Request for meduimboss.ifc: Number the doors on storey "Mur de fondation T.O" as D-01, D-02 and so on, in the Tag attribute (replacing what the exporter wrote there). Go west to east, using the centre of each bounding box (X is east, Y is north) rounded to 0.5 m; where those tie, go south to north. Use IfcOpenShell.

First a look at what the model holds.

```python
import ifcopenshell
import ifcopenshell.util.element
import ifcopenshell.util.placement

model = ifcopenshell.open("meduimboss.ifc")
print(model.schema)
storey = next(s for s in model.by_type("IfcBuildingStorey") if s.Name == "Mur de fondation T.O")
doors = [e for e in ifcopenshell.util.element.get_decomposition(storey) if e.is_a("IfcDoor")]
for e in sorted(doors, key=lambda e: e.id()):
    origin = ifcopenshell.util.placement.get_local_placement(e.ObjectPlacement)[:3, 3]
    print(e.id(), e.Tag, e.Name, origin.round(2) + 0.0, sep=" | ")
```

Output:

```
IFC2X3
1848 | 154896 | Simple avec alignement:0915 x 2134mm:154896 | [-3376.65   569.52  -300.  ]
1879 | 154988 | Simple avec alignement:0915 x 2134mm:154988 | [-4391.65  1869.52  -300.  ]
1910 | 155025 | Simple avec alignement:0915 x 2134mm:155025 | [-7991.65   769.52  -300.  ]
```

```python
import ifcopenshell
import ifcopenshell.geom
import ifcopenshell.util.element
import ifcopenshell.util.shape

model = ifcopenshell.open("meduimboss.ifc")
settings = ifcopenshell.geom.settings()
settings.set("use-world-coords", True)


def centre(element):
    shape = ifcopenshell.geom.create_shape(settings, element)
    return ifcopenshell.util.shape.get_bbox_centroid(shape.geometry)


storey = next(s for s in model.by_type("IfcBuildingStorey") if s.Name == "Mur de fondation T.O")
doors = [e for e in ifcopenshell.util.element.get_decomposition(storey) if e.is_a("IfcDoor")]

# Insertion points can sit at a corner or the storey origin, so sort by the geometry (in metres).
centres = {e: centre(e) for e in doors}
doors.sort(key=lambda e: (round(centres[e][0] / 0.5), centres[e][1]))

for i, e in enumerate(doors, start=1):
    number = f"D-{i:02d}"
    e.Tag = number
    print(e.id(), number)

model.write("meduimboss_v2.ifc")
```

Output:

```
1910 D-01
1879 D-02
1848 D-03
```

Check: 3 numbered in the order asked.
